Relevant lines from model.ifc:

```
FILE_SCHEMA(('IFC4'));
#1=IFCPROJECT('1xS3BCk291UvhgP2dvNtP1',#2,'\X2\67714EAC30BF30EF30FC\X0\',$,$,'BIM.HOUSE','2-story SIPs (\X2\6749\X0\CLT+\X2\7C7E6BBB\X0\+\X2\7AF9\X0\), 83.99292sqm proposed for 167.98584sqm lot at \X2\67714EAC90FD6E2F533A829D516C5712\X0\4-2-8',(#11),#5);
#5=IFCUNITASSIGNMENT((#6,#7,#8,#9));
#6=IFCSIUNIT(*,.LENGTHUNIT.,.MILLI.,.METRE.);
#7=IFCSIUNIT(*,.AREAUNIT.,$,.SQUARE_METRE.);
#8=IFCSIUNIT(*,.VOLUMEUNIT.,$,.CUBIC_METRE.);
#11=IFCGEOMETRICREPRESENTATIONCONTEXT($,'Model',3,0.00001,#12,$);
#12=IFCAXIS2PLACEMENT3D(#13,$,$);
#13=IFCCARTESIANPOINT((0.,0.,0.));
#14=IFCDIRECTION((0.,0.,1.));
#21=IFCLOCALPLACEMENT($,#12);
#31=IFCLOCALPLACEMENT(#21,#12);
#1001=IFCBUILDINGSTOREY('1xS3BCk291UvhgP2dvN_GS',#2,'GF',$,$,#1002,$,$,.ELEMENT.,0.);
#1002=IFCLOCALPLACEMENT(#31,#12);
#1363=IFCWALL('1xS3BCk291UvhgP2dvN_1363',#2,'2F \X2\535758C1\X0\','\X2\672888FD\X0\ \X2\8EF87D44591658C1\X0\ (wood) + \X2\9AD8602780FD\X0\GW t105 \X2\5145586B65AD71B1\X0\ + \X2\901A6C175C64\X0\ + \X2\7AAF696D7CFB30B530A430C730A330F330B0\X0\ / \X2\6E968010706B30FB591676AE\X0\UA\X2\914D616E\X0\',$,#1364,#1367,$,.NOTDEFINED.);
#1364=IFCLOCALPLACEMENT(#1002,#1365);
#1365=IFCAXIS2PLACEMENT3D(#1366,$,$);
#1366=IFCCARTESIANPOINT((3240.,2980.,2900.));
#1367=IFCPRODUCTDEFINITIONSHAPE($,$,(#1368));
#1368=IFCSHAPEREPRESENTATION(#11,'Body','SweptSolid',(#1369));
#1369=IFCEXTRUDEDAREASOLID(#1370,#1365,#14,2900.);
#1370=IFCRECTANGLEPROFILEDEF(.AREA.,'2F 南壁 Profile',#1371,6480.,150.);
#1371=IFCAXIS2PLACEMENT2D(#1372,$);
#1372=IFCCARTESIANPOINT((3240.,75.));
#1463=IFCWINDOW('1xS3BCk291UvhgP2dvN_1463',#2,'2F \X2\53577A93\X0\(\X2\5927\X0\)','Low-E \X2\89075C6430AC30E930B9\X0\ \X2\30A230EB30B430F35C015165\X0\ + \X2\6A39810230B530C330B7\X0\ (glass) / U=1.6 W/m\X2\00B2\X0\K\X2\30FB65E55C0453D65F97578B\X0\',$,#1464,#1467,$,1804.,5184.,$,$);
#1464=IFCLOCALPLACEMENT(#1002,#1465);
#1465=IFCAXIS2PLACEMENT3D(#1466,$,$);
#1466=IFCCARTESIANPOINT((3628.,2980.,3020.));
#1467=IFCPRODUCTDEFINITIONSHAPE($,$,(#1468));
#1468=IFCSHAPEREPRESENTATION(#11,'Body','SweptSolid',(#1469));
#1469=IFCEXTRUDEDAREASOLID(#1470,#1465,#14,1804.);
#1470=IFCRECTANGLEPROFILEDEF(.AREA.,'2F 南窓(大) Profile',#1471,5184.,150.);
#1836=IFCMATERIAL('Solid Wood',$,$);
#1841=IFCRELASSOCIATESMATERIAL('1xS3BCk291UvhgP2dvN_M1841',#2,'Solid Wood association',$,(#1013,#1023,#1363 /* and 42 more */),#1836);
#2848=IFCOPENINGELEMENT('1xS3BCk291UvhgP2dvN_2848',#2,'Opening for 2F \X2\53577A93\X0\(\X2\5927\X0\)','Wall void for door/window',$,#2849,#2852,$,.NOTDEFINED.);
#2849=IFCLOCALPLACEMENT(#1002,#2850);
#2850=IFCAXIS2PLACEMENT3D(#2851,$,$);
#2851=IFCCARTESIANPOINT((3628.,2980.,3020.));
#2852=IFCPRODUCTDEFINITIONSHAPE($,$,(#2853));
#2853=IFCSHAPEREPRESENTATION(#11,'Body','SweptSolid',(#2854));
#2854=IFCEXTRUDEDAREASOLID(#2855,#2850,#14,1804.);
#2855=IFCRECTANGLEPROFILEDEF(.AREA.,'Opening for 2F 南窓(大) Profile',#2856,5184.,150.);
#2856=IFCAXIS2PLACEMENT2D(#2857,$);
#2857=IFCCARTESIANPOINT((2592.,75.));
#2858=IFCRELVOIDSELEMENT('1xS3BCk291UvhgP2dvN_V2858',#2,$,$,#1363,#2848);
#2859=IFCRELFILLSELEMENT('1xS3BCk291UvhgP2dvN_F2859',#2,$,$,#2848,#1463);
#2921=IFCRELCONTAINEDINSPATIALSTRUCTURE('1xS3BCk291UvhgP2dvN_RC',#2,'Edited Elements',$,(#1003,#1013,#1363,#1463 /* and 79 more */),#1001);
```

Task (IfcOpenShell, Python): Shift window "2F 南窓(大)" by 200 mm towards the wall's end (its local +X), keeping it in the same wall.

```python
import ifcopenshell
import ifcopenshell.api.geometry
import ifcopenshell.util.placement
import ifcopenshell.util.unit

model = ifcopenshell.open("model.ifc")
unit_scale = ifcopenshell.util.unit.calculate_unit_scale(model)

window = model.by_id(1463)
opening = window.FillsVoids[0].RelatingOpeningElement
wall = opening.VoidsElements[0].RelatingBuildingElement

wall_matrix = ifcopenshell.util.placement.get_local_placement(wall.ObjectPlacement)
shift = wall_matrix[:3, 0] * 0.2 / unit_scale
before = ifcopenshell.util.placement.get_local_placement(window.ObjectPlacement)[:3, 3].copy()

# The window is not placed relative to its opening, so move both.
for product in (opening, window):
    matrix = ifcopenshell.util.placement.get_local_placement(product.ObjectPlacement)
    matrix[:3, 3] += shift
    ifcopenshell.api.geometry.edit_object_placement(model, product=product, matrix=matrix, is_si=False)

after = ifcopenshell.util.placement.get_local_placement(window.ObjectPlacement)[:3, 3]
print("window moved by", (after - before).round(3) + 0.0)

model.write("model_updated.ifc")
```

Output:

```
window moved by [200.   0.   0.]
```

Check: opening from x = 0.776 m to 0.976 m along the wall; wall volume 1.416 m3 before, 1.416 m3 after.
